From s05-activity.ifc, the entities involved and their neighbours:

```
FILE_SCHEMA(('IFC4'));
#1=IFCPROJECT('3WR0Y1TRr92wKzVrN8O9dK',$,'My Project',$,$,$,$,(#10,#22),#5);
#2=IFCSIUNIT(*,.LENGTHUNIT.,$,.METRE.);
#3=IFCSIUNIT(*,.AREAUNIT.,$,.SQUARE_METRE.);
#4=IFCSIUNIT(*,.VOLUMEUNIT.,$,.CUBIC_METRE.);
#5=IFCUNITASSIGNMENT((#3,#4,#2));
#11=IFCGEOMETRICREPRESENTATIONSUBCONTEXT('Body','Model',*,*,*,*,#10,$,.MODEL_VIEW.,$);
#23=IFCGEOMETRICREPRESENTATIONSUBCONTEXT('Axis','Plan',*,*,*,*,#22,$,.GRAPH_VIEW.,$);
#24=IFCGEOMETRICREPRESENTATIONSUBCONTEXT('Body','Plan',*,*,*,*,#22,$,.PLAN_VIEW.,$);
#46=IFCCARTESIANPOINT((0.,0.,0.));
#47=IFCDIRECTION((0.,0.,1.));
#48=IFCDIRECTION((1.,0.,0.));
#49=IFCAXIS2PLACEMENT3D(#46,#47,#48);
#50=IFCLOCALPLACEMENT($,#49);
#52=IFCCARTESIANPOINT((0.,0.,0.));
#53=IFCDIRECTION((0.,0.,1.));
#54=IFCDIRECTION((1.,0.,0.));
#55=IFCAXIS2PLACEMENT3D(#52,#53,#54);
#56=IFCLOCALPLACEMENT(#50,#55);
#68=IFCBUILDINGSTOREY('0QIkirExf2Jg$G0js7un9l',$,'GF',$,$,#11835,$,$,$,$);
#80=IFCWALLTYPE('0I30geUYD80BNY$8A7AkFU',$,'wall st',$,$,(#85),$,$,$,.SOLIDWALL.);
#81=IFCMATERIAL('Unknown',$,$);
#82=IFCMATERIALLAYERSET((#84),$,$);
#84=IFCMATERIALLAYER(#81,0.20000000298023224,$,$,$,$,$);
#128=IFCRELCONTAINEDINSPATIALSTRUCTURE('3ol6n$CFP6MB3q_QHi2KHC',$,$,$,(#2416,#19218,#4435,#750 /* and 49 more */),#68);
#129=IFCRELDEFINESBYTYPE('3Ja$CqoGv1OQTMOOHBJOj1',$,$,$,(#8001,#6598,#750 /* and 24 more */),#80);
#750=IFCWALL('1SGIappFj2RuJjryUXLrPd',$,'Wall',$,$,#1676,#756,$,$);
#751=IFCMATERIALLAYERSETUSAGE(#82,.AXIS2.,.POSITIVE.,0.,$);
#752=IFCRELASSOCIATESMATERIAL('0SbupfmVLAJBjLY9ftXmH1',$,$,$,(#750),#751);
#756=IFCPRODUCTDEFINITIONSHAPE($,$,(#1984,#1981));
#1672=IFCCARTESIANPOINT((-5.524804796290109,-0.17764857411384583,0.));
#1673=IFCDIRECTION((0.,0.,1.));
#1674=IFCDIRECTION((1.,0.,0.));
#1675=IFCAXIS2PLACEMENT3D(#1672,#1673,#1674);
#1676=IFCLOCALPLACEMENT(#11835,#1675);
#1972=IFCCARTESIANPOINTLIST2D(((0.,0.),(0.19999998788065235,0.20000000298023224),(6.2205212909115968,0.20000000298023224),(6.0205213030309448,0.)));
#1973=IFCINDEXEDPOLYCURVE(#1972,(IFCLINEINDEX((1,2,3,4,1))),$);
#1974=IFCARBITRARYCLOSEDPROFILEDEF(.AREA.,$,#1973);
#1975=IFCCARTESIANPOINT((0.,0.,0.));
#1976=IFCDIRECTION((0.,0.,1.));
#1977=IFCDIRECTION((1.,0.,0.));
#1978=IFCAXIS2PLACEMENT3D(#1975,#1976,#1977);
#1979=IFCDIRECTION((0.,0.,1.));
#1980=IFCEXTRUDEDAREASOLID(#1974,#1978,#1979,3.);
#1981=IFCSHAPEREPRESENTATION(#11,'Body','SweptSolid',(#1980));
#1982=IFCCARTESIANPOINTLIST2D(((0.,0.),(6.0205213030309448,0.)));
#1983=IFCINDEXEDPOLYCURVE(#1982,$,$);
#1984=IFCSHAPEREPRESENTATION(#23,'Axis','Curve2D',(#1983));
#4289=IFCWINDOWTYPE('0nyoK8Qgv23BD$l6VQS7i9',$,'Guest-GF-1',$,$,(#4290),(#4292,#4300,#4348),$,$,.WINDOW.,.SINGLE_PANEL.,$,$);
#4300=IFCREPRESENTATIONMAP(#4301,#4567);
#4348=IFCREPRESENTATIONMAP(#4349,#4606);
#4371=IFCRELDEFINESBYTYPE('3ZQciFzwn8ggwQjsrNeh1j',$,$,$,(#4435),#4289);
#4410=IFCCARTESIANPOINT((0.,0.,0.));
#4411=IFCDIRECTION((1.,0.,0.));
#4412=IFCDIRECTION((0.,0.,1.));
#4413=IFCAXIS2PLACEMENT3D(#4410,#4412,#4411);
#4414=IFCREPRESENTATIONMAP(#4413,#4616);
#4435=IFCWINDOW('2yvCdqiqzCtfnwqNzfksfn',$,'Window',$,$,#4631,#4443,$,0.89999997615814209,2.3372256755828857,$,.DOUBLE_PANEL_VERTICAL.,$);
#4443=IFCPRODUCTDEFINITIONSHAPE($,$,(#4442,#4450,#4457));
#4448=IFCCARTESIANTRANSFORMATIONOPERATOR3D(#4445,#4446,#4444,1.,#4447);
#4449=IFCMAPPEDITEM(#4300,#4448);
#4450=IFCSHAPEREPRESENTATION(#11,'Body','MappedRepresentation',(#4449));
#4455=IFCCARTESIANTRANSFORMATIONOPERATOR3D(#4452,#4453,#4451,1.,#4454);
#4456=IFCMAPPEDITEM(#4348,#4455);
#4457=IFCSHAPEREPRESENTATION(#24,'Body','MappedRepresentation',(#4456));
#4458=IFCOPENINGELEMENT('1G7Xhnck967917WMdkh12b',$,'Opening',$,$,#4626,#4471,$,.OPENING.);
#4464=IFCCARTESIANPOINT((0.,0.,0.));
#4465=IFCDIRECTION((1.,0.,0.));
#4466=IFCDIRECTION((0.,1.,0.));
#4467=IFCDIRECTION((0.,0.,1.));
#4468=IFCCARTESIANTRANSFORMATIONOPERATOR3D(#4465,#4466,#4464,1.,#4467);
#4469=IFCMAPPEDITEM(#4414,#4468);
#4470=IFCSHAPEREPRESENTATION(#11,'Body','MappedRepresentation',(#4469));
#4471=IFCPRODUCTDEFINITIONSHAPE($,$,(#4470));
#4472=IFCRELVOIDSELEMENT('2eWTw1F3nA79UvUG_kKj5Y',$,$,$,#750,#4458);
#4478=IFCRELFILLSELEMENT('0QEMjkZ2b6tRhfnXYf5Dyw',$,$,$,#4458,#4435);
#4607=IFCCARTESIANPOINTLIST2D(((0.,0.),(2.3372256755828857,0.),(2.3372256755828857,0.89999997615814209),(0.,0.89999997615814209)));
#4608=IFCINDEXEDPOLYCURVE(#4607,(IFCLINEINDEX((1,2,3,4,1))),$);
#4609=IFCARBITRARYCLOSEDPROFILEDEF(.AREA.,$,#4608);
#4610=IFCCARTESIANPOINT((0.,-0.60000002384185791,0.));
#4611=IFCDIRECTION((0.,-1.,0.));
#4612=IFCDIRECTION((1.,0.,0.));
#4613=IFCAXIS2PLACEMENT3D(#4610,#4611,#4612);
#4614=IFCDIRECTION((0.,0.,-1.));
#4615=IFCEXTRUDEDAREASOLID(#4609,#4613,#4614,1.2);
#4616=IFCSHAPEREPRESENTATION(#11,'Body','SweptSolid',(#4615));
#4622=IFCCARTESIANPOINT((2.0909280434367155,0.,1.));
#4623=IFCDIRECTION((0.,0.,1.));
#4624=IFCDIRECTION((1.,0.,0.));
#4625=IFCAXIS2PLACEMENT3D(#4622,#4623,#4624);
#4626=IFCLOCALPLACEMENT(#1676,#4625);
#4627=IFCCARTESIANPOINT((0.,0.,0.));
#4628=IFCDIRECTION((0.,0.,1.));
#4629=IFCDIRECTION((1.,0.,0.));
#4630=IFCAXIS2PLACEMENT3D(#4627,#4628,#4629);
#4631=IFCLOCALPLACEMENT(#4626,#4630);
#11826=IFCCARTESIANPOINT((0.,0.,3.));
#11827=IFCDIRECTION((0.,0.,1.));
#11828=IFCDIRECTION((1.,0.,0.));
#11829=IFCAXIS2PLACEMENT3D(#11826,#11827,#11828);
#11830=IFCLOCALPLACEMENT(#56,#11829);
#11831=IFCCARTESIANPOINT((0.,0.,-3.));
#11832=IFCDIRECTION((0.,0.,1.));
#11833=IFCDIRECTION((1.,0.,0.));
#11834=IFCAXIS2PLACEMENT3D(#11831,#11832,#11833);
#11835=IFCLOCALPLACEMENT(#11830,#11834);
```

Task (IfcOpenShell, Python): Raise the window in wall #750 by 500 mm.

```python
import numpy as np
import ifcopenshell
import ifcopenshell.api.geometry
import ifcopenshell.util.placement
import ifcopenshell.util.unit

model = ifcopenshell.open("s05-activity.ifc")
unit_scale = ifcopenshell.util.unit.calculate_unit_scale(model)

window = model.by_guid("2yvCdqiqzCtfnwqNzfksfn")
opening = window.FillsVoids[0].RelatingOpeningElement
dz = 0.5 / unit_scale

shift = np.array([0.0, 0.0, dz])
# The window is placed relative to its opening, so it follows when the opening moves.
matrix = ifcopenshell.util.placement.get_local_placement(opening.ObjectPlacement)
matrix[:3, 3] += shift
ifcopenshell.api.geometry.edit_object_placement(
    model, product=opening, matrix=matrix, is_si=False, should_transform_children=True
)

print(f"moved by {dz * unit_scale:+.3f} m")

model.write("s05-activity_rev.ifc")
```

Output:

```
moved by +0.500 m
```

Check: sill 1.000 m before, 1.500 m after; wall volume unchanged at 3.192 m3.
